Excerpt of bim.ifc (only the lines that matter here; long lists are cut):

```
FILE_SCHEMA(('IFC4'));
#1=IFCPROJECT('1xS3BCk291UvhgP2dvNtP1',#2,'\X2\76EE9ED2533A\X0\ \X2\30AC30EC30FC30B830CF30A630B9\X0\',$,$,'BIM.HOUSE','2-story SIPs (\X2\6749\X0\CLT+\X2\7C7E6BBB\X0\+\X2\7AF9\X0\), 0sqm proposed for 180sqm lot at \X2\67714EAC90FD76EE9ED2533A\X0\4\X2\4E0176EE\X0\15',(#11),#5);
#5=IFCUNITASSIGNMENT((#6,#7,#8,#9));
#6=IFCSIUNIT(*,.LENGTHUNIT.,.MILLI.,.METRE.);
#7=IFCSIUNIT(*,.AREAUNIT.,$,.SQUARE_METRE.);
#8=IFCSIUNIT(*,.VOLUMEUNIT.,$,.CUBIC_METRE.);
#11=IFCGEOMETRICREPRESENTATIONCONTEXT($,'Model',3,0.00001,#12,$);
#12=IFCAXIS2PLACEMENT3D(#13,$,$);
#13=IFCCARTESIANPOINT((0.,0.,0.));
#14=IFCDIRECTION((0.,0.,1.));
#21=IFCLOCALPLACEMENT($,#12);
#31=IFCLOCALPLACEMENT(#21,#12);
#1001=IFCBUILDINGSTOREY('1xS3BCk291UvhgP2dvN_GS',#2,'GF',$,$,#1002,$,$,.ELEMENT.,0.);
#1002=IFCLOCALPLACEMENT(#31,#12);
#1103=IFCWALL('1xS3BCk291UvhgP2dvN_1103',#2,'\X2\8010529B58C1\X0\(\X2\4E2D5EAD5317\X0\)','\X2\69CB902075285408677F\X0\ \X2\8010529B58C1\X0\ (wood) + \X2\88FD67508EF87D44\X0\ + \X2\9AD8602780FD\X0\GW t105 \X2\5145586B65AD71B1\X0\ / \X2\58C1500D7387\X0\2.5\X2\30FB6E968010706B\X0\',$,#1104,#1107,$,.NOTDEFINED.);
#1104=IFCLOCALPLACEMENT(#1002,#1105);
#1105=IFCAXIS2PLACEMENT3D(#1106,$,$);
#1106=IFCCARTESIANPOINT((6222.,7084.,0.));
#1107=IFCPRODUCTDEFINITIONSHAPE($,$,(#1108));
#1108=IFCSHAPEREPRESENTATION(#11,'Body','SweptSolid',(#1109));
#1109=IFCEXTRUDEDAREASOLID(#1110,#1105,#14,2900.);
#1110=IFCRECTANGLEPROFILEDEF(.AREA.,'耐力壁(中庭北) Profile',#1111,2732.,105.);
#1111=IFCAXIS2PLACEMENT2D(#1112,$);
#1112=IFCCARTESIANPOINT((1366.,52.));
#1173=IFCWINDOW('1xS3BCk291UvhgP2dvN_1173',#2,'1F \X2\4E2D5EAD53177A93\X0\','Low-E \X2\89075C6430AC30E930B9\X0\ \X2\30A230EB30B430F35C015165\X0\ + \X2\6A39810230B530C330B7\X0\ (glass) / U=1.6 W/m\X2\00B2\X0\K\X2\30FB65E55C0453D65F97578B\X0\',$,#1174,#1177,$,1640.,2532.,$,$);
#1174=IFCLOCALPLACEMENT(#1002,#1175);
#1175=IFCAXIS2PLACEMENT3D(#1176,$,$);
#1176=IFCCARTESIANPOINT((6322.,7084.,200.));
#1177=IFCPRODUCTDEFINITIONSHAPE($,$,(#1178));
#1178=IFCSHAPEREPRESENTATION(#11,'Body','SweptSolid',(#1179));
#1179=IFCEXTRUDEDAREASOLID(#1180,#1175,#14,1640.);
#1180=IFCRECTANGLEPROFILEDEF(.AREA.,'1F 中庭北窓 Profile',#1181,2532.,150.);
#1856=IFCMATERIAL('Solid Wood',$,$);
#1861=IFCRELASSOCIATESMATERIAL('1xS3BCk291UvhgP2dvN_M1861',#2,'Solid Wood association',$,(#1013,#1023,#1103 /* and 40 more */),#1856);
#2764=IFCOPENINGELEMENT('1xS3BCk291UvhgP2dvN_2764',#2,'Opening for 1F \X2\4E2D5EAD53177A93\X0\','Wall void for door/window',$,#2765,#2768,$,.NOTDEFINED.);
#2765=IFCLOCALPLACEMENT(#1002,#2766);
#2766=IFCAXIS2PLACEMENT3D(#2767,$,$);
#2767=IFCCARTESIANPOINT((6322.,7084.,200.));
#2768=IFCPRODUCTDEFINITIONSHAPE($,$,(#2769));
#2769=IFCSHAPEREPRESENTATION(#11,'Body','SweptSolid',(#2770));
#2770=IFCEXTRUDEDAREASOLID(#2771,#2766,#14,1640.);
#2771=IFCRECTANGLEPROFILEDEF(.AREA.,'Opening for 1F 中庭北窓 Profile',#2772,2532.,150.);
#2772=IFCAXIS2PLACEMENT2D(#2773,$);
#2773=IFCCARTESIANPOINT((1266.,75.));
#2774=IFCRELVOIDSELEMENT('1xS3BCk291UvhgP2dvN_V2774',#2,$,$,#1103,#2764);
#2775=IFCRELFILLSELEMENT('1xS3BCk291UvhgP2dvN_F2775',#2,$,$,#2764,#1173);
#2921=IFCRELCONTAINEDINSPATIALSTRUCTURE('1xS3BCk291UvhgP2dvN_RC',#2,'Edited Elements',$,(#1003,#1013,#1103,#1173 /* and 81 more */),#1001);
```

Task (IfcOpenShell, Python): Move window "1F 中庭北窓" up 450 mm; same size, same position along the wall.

```python
import numpy as np
import ifcopenshell
import ifcopenshell.api.geometry
import ifcopenshell.util.placement
import ifcopenshell.util.unit

model = ifcopenshell.open("bim.ifc")
unit_scale = ifcopenshell.util.unit.calculate_unit_scale(model)

window = model.by_guid("1xS3BCk291UvhgP2dvN_1173")
opening = window.FillsVoids[0].RelatingOpeningElement
dz = 0.45 / unit_scale

shift = np.array([0.0, 0.0, dz])
# The window is not placed relative to its opening, so move both.
for product in (opening, window):
    matrix = ifcopenshell.util.placement.get_local_placement(product.ObjectPlacement)
    matrix[:3, 3] += shift
    ifcopenshell.api.geometry.edit_object_placement(model, product=product, matrix=matrix, is_si=False)

print(f"moved by {dz * unit_scale:+.3f} m")

model.write("bim_edited.ifc")
```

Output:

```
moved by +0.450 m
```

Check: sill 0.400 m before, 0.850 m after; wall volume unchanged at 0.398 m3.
